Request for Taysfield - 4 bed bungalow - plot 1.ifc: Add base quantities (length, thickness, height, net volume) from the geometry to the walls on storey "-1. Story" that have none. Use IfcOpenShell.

First a look at what the model holds.

```python
import ifcopenshell
import ifcopenshell.util.element
import ifcopenshell.util.unit

model = ifcopenshell.open("Taysfield - 4 bed bungalow - plot 1.ifc")
print(model.schema)
for unit_type in ("LENGTHUNIT", "AREAUNIT", "VOLUMEUNIT"):
    print(unit_type, ifcopenshell.util.unit.calculate_unit_scale(model, unit_type))
storey = next(s for s in model.by_type("IfcBuildingStorey") if s.Name == "-1. Story")
walls = [e for e in ifcopenshell.util.element.get_decomposition(storey) if e.is_a("IfcWall")]
for e in sorted(walls, key=lambda e: e.id()):
    print(e.id(), e.is_a(), e.Name, list(ifcopenshell.util.element.get_psets(e, qtos_only=True)), sep=" | ")
```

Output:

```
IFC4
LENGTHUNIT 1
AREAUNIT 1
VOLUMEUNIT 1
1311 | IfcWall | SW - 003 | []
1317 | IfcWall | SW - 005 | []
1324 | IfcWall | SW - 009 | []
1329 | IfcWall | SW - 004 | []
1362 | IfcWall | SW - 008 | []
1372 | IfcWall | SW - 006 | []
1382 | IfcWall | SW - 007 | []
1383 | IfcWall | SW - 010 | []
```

```python
import ifcopenshell
import ifcopenshell.api.pset
import ifcopenshell.geom
import ifcopenshell.util.element
import ifcopenshell.util.shape
import ifcopenshell.util.unit

model = ifcopenshell.open("Taysfield - 4 bed bungalow - plot 1.ifc")
unit_scale = ifcopenshell.util.unit.calculate_unit_scale(model)
volume_scale = ifcopenshell.util.unit.calculate_unit_scale(model, "VOLUMEUNIT")
settings = ifcopenshell.geom.settings()

storey = next(s for s in model.by_type("IfcBuildingStorey") if s.Name == "-1. Story")
walls = [e for e in ifcopenshell.util.element.get_decomposition(storey) if e.is_a("IfcWall")]

for e in sorted(walls, key=lambda e: e.id()):
    if ifcopenshell.util.element.get_psets(e, qtos_only=True, should_inherit=False):
        continue
    # Geometry comes back in metres, in the element's own axes.
    shape = ifcopenshell.geom.create_shape(settings, e)
    values = {
        "Length": ifcopenshell.util.shape.get_x(shape.geometry) / unit_scale,
        "Width": ifcopenshell.util.shape.get_y(shape.geometry) / unit_scale,
        "Height": ifcopenshell.util.shape.get_z(shape.geometry) / unit_scale,
        "NetVolume": ifcopenshell.util.shape.get_volume(shape.geometry) / volume_scale,
    }
    qto = ifcopenshell.api.pset.add_qto(model, product=e, name="Qto_WallBaseQuantities")
    ifcopenshell.api.pset.edit_qto(model, qto=qto, properties=values)
    print(e.id(), {k: round(v, 3) for k, v in values.items()})

model.write("Taysfield - 4 bed bungalow - plot 1_edited.ifc")
```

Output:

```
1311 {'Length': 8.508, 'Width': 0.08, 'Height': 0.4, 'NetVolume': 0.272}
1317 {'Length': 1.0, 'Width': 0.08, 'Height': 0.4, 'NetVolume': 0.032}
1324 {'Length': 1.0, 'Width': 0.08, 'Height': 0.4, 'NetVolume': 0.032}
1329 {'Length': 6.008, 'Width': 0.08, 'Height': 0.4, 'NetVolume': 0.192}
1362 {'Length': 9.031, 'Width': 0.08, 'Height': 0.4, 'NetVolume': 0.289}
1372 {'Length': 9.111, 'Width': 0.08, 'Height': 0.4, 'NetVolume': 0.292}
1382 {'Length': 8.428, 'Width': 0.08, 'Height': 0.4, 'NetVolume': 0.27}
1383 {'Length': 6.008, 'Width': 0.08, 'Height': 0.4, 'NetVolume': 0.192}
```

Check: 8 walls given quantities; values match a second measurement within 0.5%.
